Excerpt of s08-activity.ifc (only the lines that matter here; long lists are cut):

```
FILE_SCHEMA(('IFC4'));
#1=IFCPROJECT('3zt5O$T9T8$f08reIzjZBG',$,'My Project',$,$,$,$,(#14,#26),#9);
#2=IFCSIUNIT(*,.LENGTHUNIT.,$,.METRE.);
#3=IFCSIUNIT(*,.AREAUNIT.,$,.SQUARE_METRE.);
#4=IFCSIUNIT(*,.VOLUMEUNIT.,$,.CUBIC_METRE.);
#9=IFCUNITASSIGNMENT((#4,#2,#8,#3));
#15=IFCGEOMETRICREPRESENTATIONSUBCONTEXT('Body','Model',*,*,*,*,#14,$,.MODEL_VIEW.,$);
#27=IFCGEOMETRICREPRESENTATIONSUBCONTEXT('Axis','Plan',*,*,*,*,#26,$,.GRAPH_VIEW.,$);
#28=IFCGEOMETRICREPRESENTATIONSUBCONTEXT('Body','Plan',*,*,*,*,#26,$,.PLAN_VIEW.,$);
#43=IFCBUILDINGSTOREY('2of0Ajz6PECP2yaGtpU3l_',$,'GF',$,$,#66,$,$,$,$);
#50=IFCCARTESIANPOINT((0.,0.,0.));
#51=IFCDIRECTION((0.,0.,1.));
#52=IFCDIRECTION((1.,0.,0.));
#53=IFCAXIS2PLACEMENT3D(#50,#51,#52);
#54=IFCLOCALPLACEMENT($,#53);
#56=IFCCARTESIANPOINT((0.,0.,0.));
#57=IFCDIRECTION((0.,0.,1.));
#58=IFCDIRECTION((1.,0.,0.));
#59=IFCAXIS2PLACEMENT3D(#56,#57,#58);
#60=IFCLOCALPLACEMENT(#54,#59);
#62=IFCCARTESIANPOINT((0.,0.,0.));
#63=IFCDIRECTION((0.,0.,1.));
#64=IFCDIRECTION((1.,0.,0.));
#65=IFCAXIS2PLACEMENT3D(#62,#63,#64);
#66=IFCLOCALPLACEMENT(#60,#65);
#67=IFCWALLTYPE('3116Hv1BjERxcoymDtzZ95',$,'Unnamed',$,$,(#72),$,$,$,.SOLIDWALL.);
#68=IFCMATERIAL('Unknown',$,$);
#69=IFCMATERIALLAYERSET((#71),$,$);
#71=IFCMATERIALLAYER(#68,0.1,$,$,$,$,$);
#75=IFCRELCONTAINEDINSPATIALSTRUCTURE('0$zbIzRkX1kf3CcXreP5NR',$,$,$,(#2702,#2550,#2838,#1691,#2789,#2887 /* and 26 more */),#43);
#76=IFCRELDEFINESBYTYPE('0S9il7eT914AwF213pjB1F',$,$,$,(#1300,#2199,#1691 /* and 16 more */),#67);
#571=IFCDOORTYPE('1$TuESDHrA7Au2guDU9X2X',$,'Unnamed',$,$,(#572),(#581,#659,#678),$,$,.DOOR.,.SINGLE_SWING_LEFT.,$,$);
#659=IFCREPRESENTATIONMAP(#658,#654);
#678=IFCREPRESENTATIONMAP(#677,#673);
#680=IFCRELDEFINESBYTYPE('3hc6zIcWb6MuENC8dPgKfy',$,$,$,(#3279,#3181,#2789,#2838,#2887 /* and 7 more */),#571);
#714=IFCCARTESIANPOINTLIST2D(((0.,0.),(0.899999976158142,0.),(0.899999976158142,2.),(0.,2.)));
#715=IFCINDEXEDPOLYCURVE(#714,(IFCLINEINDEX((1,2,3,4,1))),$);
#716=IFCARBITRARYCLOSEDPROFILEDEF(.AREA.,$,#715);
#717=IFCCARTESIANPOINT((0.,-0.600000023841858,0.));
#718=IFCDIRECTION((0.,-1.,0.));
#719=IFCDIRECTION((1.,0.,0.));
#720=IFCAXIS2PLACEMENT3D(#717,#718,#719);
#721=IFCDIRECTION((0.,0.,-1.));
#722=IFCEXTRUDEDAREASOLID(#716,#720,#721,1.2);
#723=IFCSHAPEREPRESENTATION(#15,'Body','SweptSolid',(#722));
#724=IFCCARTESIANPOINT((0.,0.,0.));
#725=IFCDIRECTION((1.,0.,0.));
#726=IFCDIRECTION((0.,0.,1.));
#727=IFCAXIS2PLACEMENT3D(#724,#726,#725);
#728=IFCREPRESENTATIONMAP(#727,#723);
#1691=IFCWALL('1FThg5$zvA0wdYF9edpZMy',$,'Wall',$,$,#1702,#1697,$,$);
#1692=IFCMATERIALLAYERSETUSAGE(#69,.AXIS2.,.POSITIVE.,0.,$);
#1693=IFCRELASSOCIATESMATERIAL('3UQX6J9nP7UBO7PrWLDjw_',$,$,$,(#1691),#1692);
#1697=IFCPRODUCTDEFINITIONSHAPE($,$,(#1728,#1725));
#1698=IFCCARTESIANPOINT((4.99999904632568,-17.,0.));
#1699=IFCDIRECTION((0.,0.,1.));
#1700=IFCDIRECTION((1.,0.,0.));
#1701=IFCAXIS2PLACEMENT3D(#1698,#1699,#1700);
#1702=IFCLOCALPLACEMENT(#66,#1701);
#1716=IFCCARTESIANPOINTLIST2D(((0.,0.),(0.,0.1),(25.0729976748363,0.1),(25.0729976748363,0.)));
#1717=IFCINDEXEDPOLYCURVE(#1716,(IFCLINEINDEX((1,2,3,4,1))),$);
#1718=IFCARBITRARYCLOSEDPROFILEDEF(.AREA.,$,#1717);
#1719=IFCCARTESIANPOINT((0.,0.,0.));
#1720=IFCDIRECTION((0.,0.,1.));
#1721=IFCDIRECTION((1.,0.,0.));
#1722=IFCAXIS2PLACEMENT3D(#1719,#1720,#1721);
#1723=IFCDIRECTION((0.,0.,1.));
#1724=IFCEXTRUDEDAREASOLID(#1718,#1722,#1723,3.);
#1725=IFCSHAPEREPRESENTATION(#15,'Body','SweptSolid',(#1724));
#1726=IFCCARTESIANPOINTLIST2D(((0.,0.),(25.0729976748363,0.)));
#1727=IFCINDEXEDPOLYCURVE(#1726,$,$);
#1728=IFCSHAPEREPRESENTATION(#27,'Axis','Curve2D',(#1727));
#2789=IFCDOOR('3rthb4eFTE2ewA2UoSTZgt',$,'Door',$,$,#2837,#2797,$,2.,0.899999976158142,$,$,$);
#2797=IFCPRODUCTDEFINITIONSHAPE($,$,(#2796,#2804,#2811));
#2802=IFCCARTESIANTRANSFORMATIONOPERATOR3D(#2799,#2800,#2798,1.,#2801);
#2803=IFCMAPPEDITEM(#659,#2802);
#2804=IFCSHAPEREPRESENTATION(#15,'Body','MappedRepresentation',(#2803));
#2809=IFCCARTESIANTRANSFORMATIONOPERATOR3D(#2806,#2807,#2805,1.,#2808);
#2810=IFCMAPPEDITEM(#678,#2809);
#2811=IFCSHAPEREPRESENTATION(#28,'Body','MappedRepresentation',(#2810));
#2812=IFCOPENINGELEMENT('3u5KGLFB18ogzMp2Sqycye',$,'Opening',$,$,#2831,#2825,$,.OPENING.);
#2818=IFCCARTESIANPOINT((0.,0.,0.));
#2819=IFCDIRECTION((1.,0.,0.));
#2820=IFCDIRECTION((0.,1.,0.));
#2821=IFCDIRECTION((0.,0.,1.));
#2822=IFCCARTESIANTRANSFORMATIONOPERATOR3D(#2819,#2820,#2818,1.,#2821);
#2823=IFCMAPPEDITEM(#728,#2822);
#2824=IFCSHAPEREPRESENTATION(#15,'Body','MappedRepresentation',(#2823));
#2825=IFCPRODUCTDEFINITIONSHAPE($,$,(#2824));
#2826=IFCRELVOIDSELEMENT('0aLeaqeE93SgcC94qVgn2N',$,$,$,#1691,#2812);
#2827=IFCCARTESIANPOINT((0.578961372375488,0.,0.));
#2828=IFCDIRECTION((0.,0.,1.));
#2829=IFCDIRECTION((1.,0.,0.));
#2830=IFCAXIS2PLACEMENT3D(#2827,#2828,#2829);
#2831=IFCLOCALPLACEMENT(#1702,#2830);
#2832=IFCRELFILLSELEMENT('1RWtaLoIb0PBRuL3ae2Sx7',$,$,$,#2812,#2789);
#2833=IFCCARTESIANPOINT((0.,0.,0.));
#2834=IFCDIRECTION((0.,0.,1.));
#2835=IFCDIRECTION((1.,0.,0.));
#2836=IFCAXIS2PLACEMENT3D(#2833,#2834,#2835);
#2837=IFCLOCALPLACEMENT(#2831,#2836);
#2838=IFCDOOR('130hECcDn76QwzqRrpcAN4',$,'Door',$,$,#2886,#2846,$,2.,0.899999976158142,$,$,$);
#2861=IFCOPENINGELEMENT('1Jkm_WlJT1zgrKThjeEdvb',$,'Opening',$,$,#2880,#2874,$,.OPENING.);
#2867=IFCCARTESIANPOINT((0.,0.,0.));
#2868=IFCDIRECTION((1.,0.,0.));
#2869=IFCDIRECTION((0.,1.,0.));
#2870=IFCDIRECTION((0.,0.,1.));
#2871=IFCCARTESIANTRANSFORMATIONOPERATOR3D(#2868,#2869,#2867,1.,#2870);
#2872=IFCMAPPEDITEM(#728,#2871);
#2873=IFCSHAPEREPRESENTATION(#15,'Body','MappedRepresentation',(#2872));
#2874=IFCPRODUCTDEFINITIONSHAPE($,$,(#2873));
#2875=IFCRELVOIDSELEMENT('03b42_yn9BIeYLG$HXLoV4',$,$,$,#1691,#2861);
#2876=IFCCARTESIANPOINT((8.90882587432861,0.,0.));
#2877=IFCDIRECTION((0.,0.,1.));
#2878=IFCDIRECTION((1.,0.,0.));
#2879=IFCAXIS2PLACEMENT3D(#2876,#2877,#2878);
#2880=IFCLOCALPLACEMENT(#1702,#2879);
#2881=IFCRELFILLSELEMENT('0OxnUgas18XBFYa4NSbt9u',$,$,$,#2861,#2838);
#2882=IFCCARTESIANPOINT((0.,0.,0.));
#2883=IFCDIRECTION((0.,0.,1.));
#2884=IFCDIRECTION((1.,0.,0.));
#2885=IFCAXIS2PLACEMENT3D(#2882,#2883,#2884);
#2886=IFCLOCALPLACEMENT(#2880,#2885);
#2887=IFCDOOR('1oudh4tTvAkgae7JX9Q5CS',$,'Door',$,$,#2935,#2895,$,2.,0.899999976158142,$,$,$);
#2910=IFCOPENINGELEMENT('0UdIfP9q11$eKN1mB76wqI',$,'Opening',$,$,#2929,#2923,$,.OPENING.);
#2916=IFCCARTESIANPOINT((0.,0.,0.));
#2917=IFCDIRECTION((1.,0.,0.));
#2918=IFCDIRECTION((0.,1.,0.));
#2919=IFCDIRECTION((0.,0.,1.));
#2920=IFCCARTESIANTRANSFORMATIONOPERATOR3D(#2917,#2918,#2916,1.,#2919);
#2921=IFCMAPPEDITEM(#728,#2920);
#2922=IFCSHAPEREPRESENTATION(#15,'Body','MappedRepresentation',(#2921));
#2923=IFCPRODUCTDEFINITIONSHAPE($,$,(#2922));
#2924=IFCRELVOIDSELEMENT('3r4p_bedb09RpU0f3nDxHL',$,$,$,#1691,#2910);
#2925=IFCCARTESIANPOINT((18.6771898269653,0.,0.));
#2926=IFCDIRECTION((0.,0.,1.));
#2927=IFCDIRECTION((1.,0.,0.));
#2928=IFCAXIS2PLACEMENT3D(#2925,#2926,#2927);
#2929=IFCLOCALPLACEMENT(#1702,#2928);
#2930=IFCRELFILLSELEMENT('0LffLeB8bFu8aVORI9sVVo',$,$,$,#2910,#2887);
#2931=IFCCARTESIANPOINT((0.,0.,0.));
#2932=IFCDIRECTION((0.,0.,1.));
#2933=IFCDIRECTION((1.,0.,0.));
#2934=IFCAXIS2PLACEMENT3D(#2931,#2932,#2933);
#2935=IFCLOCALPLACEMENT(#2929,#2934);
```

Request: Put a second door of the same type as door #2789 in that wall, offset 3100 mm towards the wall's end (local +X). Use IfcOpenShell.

```python
import ifcopenshell
import ifcopenshell.api.feature
import ifcopenshell.api.geometry
import ifcopenshell.api.root
import ifcopenshell.geom
import ifcopenshell.util.element
import ifcopenshell.util.placement
import ifcopenshell.util.shape

model = ifcopenshell.open("s08-activity.ifc")
settings = ifcopenshell.geom.settings()


def volume(element):
    """Net volume in cubic metres, openings subtracted."""
    shape = ifcopenshell.geom.create_shape(settings, element)
    return ifcopenshell.util.shape.get_volume(shape.geometry)


door = model.by_guid("3rthb4eFTE2ewA2UoSTZgt")
opening = door.FillsVoids[0].RelatingOpeningElement
wall = opening.VoidsElements[0].RelatingBuildingElement
before = volume(wall)
shift = ifcopenshell.util.placement.get_local_placement(wall.ObjectPlacement)[:3, 0] * 3.1

# copy_class copies the void relationship, type, container and properties, but no geometry.
new_opening = ifcopenshell.api.root.copy_class(model, product=opening)
new_opening.Representation = ifcopenshell.util.element.copy_deep(
    model, opening.Representation, exclude=["IfcGeometricRepresentationContext", "IfcRepresentationMap"]
)
new_door = ifcopenshell.api.root.copy_class(model, product=door)
new_door.Representation = ifcopenshell.util.element.copy_deep(
    model, door.Representation, exclude=["IfcGeometricRepresentationContext", "IfcRepresentationMap"]
)
ifcopenshell.api.feature.add_filling(model, opening=new_opening, element=new_door)

for old, new in ((opening, new_opening), (door, new_door)):
    matrix = ifcopenshell.util.placement.get_local_placement(old.ObjectPlacement)
    matrix[:3, 3] += shift
    ifcopenshell.api.geometry.edit_object_placement(model, product=new, matrix=matrix, is_si=False)

after = volume(wall)

print(f"wall volume {before:.3f} -> {after:.3f} m3")

model.write("s08-activity_v2.ifc")
```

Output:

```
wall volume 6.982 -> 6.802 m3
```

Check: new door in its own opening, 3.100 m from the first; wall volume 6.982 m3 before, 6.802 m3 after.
